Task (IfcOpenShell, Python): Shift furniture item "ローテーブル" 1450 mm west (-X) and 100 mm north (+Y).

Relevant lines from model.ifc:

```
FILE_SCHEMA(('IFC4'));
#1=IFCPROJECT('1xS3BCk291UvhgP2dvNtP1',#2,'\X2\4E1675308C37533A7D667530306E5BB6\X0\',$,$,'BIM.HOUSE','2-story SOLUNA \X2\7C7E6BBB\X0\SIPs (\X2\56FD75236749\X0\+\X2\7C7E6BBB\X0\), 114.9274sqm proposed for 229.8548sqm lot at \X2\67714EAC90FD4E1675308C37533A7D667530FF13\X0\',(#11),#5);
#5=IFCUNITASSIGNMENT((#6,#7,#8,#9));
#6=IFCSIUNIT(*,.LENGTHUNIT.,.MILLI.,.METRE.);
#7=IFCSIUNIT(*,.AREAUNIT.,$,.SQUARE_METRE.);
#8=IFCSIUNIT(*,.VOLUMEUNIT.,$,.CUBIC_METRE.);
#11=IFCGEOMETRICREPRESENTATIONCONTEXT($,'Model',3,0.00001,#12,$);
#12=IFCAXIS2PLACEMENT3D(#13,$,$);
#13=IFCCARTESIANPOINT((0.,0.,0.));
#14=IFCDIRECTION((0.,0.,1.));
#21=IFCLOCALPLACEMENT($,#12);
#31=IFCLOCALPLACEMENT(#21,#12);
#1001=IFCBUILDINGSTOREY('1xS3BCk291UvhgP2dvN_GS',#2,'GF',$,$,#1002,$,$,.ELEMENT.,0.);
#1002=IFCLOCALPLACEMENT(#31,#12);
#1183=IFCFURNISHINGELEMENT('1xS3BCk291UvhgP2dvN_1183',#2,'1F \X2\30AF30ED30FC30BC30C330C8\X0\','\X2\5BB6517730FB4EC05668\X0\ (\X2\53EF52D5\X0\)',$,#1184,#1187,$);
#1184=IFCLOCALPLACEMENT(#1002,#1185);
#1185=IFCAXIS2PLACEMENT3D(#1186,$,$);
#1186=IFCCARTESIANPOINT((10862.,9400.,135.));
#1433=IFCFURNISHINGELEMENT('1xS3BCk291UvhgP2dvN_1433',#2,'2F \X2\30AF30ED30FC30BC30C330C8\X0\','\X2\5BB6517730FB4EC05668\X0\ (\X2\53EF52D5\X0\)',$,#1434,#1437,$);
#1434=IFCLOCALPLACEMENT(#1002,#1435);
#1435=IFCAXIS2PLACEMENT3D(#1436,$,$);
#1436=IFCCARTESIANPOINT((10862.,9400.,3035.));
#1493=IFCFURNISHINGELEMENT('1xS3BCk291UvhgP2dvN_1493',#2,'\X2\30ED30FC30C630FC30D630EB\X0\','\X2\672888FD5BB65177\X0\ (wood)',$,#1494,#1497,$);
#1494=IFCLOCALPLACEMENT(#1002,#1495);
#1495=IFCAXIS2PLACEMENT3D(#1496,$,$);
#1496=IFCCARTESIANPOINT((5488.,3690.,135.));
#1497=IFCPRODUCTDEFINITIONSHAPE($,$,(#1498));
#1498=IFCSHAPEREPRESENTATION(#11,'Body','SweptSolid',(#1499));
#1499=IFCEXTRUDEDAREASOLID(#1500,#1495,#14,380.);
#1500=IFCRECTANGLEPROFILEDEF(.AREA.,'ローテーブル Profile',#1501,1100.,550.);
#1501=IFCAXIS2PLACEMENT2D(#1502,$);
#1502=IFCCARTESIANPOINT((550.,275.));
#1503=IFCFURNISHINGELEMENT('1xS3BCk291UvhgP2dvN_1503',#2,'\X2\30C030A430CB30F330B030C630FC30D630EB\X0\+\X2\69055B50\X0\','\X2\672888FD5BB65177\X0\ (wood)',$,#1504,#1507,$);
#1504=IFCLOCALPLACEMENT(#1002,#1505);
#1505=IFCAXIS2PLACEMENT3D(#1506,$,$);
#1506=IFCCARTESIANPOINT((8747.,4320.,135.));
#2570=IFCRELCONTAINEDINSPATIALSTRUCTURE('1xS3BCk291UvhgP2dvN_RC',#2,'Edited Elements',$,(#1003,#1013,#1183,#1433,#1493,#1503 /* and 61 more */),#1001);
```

```python
import ifcopenshell
import ifcopenshell.api.geometry
import ifcopenshell.util.placement
import ifcopenshell.util.unit

model = ifcopenshell.open("model.ifc")
unit_scale = ifcopenshell.util.unit.calculate_unit_scale(model)

item = model.by_guid("1xS3BCk291UvhgP2dvN_1493")
matrix = ifcopenshell.util.placement.get_local_placement(item.ObjectPlacement)
matrix[0, 3] -= 1.45 / unit_scale
matrix[1, 3] += 0.1 / unit_scale
ifcopenshell.api.geometry.edit_object_placement(model, product=item, matrix=matrix, is_si=False)

print(ifcopenshell.util.placement.get_local_placement(item.ObjectPlacement).round(3) + 0.0)

model.write("model-out.ifc")
```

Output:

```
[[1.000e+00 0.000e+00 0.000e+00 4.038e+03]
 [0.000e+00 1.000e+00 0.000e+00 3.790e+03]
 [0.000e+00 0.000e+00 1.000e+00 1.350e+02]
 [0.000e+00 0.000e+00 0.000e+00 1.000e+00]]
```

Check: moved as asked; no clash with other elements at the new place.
